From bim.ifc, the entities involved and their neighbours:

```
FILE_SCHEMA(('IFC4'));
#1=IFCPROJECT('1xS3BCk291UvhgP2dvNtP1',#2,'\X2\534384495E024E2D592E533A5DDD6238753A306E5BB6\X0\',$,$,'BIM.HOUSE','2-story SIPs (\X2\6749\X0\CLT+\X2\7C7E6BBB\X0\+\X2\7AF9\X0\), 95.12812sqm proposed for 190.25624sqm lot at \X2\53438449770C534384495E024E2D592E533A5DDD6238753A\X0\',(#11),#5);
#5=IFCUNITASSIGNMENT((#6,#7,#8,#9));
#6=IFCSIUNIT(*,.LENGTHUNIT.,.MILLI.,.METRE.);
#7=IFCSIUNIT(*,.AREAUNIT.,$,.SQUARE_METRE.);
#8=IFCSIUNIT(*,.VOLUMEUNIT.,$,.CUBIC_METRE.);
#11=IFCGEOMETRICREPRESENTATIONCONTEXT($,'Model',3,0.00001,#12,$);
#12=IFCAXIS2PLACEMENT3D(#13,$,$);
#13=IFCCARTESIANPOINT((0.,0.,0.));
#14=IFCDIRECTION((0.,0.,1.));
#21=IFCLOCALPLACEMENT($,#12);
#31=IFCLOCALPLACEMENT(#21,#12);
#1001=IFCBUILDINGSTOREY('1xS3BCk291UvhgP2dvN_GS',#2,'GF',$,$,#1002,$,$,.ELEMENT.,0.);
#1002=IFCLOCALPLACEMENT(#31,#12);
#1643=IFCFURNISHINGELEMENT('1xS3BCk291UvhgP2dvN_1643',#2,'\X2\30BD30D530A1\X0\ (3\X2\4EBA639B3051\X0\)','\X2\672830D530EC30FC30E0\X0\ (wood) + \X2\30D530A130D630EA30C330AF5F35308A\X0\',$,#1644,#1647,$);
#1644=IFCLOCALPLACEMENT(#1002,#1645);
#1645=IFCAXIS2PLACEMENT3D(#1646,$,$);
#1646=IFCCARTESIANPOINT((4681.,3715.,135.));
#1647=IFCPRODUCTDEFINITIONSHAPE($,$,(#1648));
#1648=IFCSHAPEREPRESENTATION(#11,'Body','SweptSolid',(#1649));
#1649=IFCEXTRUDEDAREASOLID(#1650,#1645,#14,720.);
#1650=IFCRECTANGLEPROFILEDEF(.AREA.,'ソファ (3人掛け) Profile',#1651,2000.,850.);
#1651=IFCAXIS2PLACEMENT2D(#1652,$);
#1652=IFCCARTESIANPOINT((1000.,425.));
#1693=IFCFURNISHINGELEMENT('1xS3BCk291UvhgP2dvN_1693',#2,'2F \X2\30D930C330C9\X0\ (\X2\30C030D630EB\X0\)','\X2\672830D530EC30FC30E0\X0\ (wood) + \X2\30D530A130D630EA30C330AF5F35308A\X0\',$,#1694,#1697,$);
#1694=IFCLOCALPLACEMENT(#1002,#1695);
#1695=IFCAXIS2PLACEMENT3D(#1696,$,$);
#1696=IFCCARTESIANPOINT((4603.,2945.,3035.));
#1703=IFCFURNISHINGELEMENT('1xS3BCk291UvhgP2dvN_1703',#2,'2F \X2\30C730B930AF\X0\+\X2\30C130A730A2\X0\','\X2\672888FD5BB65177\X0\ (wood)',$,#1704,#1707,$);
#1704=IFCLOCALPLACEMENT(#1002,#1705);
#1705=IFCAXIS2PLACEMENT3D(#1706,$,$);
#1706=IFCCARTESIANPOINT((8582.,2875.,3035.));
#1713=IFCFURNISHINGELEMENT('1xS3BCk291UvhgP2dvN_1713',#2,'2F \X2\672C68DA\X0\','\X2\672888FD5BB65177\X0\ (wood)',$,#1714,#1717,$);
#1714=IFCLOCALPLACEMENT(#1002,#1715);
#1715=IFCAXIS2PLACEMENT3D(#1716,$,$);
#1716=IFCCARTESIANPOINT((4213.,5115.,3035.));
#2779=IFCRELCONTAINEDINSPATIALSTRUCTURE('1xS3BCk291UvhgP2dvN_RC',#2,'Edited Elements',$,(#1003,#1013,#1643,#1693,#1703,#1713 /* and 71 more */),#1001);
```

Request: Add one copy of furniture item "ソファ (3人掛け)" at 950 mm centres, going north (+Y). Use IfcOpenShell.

```python
import numpy as np
import ifcopenshell
import ifcopenshell.api.geometry
import ifcopenshell.api.root
import ifcopenshell.util.element
import ifcopenshell.util.placement

model = ifcopenshell.open("bim.ifc")


def reuse_history(source, copy):
    """copy_class also copies each property set's owner history, people and application; keep the originals."""
    for rel in copy.IsDefinedBy:
        if rel.is_a("IfcRelDefinesByProperties") and (history := rel.RelatingPropertyDefinition.OwnerHistory):
            rel.RelatingPropertyDefinition.OwnerHistory = source.OwnerHistory
            ifcopenshell.util.element.remove_deep2(model, history)


source = model.by_guid("1xS3BCk291UvhgP2dvN_1643")
base = ifcopenshell.util.placement.get_local_placement(source.ObjectPlacement)
step = np.array([0.0, 1.0, 0.0]) * 950.0

for i in range(1, 2):
    copy = ifcopenshell.api.root.copy_class(model, product=source)
    copy.Representation = ifcopenshell.util.element.copy_deep(
        model, source.Representation, exclude=["IfcGeometricRepresentationContext", "IfcRepresentationMap"]
    )
    reuse_history(source, copy)
    matrix = base.copy()
    matrix[:3, 3] += i * step
    print("added at", matrix[:3, 3].round(3) + 0.0)
    ifcopenshell.api.geometry.edit_object_placement(model, product=copy, matrix=matrix, is_si=False)

model.write("bim_edited.ifc")
```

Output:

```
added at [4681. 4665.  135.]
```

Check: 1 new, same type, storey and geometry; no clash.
